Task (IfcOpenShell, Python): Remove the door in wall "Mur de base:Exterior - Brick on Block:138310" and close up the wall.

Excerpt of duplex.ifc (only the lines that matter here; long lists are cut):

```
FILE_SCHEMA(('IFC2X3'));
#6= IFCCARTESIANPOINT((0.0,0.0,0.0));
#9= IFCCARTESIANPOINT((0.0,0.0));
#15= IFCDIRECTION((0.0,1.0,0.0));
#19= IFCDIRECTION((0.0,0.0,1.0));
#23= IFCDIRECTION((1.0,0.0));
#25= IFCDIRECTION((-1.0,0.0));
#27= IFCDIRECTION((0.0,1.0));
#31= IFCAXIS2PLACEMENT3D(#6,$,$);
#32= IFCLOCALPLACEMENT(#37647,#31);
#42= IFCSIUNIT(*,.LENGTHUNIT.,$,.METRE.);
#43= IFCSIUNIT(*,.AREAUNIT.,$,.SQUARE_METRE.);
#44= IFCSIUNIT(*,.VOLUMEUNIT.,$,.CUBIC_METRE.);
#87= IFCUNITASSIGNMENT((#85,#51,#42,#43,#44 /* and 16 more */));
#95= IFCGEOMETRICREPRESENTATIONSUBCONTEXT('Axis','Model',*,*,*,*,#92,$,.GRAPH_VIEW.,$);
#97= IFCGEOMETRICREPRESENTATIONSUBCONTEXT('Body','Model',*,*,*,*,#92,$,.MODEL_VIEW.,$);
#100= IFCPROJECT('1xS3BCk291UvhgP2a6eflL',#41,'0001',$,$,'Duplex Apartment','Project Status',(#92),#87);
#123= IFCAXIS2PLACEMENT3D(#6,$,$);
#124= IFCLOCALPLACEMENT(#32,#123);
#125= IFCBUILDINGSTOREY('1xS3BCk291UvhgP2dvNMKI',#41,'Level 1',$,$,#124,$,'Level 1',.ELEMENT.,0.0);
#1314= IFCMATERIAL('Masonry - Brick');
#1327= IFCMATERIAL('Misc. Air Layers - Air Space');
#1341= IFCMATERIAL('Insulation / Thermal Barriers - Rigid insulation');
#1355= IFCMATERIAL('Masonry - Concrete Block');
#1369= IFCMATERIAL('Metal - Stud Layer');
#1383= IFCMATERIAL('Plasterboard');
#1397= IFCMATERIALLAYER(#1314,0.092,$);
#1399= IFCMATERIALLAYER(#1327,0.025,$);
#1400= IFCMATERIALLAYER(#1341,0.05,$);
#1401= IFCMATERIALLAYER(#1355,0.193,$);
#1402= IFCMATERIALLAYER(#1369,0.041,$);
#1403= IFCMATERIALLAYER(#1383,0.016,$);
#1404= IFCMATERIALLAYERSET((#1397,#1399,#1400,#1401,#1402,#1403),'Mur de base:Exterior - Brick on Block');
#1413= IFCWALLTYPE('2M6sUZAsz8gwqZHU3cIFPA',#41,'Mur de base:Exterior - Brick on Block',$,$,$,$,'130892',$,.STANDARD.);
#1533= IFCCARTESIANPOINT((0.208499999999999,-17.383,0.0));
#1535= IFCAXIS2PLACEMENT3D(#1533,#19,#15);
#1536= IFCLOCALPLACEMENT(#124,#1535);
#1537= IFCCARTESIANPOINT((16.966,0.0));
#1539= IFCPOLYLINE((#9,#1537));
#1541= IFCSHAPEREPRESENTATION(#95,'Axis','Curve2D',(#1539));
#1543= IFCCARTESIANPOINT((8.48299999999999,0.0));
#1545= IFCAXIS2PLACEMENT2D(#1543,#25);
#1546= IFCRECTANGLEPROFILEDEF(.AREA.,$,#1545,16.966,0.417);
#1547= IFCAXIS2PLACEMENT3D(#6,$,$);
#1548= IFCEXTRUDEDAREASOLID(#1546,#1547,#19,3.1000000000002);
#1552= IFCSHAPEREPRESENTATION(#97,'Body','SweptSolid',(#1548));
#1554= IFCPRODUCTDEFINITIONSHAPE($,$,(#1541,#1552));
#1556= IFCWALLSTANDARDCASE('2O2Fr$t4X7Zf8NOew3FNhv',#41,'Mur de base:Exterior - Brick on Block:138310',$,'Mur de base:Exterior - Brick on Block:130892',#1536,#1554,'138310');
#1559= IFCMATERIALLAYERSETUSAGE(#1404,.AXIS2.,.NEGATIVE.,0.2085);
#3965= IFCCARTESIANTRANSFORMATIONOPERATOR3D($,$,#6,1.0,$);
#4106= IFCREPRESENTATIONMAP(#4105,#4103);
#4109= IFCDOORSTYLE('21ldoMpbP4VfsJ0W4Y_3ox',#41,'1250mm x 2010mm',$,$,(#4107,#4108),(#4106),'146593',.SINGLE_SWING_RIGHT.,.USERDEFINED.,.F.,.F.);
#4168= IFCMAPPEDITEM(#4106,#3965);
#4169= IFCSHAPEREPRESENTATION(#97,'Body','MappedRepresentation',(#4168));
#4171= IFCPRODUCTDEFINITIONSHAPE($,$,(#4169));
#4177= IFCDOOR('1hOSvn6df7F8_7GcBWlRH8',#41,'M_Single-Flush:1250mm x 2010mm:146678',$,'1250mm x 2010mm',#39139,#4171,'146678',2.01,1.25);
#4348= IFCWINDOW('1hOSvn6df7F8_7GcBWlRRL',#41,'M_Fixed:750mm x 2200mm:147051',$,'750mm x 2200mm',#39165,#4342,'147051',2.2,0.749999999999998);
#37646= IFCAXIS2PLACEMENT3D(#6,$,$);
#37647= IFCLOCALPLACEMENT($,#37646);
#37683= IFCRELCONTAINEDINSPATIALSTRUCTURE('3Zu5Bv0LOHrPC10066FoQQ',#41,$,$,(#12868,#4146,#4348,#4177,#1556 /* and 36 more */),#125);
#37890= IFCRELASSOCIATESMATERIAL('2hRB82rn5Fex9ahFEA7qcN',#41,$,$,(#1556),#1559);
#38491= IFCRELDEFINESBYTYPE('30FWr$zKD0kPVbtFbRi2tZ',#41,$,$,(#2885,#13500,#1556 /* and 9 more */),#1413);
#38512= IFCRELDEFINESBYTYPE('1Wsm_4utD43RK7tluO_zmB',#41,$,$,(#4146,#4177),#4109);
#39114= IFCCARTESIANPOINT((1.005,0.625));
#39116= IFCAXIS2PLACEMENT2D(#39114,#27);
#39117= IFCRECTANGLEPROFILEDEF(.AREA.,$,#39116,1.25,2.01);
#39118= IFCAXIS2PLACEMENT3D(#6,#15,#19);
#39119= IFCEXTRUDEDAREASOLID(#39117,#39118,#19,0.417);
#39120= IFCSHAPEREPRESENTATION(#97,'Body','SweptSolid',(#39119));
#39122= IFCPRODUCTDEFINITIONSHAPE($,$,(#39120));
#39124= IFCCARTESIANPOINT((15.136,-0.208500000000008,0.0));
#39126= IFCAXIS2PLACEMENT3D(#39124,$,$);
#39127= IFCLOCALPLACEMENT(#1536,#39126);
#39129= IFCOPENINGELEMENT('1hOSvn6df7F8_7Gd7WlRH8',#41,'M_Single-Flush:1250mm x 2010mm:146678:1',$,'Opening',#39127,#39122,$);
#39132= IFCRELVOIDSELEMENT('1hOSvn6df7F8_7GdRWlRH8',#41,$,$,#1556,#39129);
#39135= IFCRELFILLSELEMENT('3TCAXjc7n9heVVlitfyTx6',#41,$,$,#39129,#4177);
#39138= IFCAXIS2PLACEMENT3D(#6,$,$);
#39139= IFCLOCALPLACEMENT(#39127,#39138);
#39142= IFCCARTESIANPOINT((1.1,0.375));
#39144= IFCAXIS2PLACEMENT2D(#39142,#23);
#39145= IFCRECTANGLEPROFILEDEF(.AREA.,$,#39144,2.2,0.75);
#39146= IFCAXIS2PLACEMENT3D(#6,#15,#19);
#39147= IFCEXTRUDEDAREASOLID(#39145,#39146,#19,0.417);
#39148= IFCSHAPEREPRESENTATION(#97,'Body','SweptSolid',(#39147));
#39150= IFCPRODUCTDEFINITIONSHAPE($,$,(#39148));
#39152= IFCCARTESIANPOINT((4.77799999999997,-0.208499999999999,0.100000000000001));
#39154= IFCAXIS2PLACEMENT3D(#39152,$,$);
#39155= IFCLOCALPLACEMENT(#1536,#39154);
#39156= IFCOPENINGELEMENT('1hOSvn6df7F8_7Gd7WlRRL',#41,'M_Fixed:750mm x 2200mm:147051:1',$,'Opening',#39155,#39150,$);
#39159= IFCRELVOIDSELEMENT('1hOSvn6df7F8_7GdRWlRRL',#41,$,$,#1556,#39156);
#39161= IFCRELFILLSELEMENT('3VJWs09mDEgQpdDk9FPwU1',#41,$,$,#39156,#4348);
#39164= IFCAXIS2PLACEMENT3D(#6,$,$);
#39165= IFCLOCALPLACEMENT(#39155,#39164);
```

```python
import ifcopenshell
import ifcopenshell.api.feature
import ifcopenshell.api.root
import ifcopenshell.geom
import ifcopenshell.util.shape

model = ifcopenshell.open("duplex.ifc")
settings = ifcopenshell.geom.settings()


def volume(element):
    """Net volume in cubic metres, openings subtracted."""
    shape = ifcopenshell.geom.create_shape(settings, element)
    return ifcopenshell.util.shape.get_volume(shape.geometry)


door = model.by_guid("1hOSvn6df7F8_7GcBWlRH8")
opening = door.FillsVoids[0].RelatingOpeningElement
wall = opening.VoidsElements[0].RelatingBuildingElement
before = volume(wall)

ifcopenshell.api.root.remove_product(model, product=door)
ifcopenshell.api.feature.remove_feature(model, feature=opening)

after = volume(wall)

print(f"wall volume {before:.3f} -> {after:.3f} m3")

model.write("duplex-out.ifc")
```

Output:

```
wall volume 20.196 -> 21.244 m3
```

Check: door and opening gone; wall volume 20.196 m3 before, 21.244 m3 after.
